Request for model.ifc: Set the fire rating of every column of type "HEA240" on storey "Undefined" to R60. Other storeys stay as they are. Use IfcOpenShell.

First a look at what the model holds.

```python
import ifcopenshell
import ifcopenshell.util.element

model = ifcopenshell.open("model.ifc")
print(model.schema)
storey = next(s for s in model.by_type("IfcBuildingStorey") if s.Name == "Undefined")
columns = [e for e in ifcopenshell.util.element.get_decomposition(storey) if e.is_a("IfcColumn")]
seen = {}
for e in columns:
    element_type = ifcopenshell.util.element.get_type(e)
    key = (element_type.Name if element_type != e and element_type else None, ifcopenshell.util.element.get_pset(e, "Pset_ColumnCommon", "FireRating"))
    seen[key] = seen.get(key, 0) + 1
for (name, value), count in sorted(seen.items(), key=str):
    print(count, "x", name, "|", value)
```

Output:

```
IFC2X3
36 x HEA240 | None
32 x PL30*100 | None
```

```python
import ifcopenshell
import ifcopenshell.api.pset
import ifcopenshell.util.element

model = ifcopenshell.open("model.ifc")

storey = next(s for s in model.by_type("IfcBuildingStorey") if s.Name == "Undefined")
columns = [e for e in ifcopenshell.util.element.get_decomposition(storey) if e.is_a("IfcColumn")]

count = 0
for e in columns:
    element_type = ifcopenshell.util.element.get_type(e)
    if element_type in (None, e) or element_type.Name != "HEA240":
        continue
    # add_pset returns the element's existing set when there is one.
    pset = ifcopenshell.api.pset.add_pset(model, product=e, name="Pset_ColumnCommon")
    ifcopenshell.api.pset.edit_pset(model, pset=pset, properties={"FireRating": "R60"})
    count += 1

print(count, "columns updated")

model.write("model_v2.ifc")
```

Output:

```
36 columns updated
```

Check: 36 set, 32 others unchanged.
